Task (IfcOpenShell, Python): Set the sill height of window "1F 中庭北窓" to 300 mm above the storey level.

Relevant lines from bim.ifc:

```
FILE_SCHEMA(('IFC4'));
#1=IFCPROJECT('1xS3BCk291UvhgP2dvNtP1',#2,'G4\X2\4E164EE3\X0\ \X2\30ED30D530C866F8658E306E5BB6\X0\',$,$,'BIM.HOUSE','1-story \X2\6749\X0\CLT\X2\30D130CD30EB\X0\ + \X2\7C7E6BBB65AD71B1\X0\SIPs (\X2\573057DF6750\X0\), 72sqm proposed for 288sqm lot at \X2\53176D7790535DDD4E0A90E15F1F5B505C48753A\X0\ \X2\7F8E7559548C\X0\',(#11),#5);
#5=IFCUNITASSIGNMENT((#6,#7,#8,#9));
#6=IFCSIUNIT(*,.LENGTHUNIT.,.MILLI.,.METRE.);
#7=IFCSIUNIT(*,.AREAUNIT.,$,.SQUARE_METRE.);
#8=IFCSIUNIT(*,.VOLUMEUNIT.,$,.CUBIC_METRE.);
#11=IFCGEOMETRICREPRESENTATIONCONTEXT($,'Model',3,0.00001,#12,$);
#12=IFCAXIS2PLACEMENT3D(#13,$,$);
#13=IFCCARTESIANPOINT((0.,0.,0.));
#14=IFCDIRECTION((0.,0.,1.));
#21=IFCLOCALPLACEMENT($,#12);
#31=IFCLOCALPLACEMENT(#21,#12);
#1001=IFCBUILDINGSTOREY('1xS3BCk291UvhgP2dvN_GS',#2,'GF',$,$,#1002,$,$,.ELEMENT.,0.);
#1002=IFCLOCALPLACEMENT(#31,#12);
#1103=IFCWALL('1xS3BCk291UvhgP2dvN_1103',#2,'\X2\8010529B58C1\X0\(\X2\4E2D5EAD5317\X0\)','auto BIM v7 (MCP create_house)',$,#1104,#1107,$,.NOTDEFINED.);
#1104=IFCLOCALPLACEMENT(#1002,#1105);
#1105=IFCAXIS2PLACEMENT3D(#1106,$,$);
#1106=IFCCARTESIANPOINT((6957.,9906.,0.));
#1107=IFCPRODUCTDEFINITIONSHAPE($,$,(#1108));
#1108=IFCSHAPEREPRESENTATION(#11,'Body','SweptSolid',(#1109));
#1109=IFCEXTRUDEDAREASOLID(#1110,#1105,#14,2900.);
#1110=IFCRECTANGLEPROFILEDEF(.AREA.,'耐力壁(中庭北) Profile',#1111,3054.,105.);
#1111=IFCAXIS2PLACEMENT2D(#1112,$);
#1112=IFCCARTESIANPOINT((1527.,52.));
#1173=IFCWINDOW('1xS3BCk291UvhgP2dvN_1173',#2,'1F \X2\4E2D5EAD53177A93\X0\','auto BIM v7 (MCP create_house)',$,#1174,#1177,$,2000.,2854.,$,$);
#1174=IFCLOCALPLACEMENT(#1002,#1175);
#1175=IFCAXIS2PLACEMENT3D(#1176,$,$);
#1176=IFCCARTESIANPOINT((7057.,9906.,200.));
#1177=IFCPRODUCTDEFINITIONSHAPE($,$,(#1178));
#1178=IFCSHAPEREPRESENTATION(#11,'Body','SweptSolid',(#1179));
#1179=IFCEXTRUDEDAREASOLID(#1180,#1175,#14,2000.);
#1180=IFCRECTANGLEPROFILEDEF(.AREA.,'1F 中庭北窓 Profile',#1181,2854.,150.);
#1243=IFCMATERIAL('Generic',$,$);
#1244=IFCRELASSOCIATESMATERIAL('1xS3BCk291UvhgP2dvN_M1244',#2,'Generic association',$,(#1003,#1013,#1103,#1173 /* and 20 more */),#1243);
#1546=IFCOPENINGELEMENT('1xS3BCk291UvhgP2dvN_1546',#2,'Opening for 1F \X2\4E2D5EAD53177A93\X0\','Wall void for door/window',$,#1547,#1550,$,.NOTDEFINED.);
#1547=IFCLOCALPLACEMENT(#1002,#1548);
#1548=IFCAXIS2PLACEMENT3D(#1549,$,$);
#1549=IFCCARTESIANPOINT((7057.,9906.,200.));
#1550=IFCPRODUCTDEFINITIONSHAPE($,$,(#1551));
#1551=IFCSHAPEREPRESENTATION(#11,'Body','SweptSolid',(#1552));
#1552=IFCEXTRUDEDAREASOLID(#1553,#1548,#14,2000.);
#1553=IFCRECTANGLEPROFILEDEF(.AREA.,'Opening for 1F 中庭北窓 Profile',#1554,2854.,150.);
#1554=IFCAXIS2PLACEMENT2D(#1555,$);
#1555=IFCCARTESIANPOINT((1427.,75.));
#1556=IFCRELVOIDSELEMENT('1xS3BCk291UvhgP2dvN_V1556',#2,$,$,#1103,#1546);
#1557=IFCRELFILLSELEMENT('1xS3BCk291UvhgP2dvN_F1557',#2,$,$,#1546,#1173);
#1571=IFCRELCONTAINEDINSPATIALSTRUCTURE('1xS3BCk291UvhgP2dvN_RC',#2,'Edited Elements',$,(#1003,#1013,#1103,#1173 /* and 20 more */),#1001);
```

```python
import numpy as np
import ifcopenshell
import ifcopenshell.api.geometry
import ifcopenshell.geom
import ifcopenshell.util.element
import ifcopenshell.util.placement
import ifcopenshell.util.shape
import ifcopenshell.util.unit

model = ifcopenshell.open("bim.ifc")
unit_scale = ifcopenshell.util.unit.calculate_unit_scale(model)

window = model.by_id(1173)
opening = window.FillsVoids[0].RelatingOpeningElement
storey = ifcopenshell.util.element.get_container(window, ifc_class="IfcBuildingStorey")
level = ifcopenshell.util.placement.get_local_placement(storey.ObjectPlacement)[2, 3]

# The opening's origin need not be at the sill, so measure its lowest point.
shape = ifcopenshell.geom.create_shape(ifcopenshell.geom.settings(), opening)
bottom = ifcopenshell.util.shape.get_shape_bottom_elevation(shape, shape.geometry) / unit_scale
dz = level + 0.3 / unit_scale - bottom

shift = np.array([0.0, 0.0, dz])
# The window is not placed relative to its opening, so move both.
for product in (opening, window):
    matrix = ifcopenshell.util.placement.get_local_placement(product.ObjectPlacement)
    matrix[:3, 3] += shift
    ifcopenshell.api.geometry.edit_object_placement(model, product=product, matrix=matrix, is_si=False)

print(f"moved by {dz * unit_scale:+.3f} m")

model.write("bim_v2.ifc")
```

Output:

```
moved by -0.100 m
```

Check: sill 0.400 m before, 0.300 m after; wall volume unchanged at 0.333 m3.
